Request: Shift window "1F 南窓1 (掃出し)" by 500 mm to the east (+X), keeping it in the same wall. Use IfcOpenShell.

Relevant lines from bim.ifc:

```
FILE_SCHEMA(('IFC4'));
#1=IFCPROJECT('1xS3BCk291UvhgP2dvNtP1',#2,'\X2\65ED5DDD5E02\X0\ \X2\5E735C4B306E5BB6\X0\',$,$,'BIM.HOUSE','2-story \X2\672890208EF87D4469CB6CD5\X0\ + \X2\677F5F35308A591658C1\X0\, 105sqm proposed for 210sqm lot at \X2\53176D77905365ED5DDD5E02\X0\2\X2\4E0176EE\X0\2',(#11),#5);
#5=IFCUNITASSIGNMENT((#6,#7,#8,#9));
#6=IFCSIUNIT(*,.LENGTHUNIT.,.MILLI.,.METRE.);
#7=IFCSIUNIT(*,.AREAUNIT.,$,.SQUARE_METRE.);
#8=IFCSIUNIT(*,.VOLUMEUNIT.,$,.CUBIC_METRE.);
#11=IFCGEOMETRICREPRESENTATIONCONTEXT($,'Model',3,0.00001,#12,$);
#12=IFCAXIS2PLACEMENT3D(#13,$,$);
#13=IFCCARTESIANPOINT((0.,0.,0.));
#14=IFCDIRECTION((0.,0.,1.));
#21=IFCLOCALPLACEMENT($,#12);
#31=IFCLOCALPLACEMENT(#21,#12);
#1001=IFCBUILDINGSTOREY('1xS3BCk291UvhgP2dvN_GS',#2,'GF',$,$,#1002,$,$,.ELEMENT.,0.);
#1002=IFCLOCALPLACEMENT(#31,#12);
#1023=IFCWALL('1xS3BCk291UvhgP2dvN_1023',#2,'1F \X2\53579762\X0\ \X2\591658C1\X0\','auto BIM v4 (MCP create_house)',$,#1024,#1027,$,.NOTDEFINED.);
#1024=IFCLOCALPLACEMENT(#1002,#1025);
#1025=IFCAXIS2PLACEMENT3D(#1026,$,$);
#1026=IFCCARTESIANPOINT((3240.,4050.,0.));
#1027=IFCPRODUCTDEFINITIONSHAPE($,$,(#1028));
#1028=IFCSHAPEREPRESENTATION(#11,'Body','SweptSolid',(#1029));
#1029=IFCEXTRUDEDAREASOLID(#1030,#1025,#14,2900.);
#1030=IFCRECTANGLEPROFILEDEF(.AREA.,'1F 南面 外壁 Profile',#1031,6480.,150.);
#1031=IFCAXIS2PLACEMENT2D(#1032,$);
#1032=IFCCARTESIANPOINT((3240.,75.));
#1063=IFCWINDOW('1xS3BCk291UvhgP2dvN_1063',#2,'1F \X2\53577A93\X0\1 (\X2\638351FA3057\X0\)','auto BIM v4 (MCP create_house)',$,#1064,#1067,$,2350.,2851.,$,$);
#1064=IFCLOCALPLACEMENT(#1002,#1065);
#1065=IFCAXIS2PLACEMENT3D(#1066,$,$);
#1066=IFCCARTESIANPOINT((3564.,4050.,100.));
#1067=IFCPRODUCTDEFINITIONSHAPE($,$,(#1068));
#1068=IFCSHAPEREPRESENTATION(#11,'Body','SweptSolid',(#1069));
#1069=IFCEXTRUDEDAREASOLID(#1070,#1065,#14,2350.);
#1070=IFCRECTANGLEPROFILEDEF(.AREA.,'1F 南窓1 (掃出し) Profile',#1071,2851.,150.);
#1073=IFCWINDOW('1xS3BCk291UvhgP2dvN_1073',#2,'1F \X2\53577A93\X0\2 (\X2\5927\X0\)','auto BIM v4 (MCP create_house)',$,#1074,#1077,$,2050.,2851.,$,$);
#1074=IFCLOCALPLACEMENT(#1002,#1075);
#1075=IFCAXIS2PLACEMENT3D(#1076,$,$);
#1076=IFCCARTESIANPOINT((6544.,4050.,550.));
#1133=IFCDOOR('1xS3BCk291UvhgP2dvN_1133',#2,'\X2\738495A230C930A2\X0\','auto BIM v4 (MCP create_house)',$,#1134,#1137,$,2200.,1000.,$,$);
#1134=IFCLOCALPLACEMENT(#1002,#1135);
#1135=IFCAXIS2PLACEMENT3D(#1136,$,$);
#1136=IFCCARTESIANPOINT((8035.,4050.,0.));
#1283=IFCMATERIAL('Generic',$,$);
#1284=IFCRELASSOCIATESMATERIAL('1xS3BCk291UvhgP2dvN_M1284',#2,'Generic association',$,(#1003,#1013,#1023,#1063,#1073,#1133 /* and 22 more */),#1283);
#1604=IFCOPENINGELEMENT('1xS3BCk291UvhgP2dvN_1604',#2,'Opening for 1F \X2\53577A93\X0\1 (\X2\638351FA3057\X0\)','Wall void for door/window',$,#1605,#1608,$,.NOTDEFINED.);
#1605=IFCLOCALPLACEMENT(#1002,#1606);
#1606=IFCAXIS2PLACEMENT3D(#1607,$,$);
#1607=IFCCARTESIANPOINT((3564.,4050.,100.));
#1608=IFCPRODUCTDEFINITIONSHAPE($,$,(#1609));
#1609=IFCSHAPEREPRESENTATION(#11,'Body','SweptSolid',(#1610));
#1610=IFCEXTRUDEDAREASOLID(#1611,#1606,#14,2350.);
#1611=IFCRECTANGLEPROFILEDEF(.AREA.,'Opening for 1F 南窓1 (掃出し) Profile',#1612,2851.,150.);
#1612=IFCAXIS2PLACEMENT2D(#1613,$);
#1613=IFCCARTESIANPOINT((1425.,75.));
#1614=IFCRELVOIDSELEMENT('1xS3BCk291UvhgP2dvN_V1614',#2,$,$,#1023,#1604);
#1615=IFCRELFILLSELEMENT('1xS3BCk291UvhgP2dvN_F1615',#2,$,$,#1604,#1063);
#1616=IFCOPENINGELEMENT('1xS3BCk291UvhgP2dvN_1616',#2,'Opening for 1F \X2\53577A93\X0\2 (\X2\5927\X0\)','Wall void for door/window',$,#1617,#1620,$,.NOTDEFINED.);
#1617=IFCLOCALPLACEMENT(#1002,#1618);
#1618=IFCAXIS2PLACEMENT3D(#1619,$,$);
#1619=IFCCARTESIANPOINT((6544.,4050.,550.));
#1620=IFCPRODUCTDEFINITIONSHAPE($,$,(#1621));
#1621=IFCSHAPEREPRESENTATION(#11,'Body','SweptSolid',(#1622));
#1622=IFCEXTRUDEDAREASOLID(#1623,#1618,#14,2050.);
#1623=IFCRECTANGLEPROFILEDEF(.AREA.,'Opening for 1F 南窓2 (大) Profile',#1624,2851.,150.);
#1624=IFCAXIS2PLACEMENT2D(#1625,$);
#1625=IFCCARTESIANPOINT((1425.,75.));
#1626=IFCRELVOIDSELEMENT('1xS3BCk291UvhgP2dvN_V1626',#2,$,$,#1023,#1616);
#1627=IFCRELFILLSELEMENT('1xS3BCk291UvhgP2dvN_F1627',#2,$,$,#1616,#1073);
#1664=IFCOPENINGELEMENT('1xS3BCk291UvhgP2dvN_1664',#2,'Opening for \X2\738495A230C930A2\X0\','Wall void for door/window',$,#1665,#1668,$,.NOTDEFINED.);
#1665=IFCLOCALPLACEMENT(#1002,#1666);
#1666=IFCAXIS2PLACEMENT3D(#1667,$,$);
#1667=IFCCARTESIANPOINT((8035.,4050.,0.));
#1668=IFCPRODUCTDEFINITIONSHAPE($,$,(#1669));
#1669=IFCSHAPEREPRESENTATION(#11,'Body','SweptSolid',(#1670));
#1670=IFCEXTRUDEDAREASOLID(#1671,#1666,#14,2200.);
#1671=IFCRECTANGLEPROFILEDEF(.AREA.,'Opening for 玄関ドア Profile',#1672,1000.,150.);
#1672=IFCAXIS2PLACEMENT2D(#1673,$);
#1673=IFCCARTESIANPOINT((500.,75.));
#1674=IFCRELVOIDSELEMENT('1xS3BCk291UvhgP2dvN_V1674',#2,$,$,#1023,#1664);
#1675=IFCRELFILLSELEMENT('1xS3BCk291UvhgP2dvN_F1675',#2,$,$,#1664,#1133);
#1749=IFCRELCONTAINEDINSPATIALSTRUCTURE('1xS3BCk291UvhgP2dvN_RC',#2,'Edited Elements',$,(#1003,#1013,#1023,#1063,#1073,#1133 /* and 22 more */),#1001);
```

```python
import ifcopenshell
import ifcopenshell.api.geometry
import ifcopenshell.util.placement

model = ifcopenshell.open("bim.ifc")

window = model.by_id(1063)
opening = window.FillsVoids[0].RelatingOpeningElement
wall = opening.VoidsElements[0].RelatingBuildingElement

wall_matrix = ifcopenshell.util.placement.get_local_placement(wall.ObjectPlacement)
shift = wall_matrix[:3, 0] * 500.0
before = ifcopenshell.util.placement.get_local_placement(window.ObjectPlacement)[:3, 3].copy()

# The window is not placed relative to its opening, so move both.
for product in (opening, window):
    matrix = ifcopenshell.util.placement.get_local_placement(product.ObjectPlacement)
    matrix[:3, 3] += shift
    ifcopenshell.api.geometry.edit_object_placement(model, product=product, matrix=matrix, is_si=False)

after = ifcopenshell.util.placement.get_local_placement(window.ObjectPlacement)[:3, 3]
print("window moved by", (after - before).round(3) + 0.0)

model.write("bim-out.ifc")
```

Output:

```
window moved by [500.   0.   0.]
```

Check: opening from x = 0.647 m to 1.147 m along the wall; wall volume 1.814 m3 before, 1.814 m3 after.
